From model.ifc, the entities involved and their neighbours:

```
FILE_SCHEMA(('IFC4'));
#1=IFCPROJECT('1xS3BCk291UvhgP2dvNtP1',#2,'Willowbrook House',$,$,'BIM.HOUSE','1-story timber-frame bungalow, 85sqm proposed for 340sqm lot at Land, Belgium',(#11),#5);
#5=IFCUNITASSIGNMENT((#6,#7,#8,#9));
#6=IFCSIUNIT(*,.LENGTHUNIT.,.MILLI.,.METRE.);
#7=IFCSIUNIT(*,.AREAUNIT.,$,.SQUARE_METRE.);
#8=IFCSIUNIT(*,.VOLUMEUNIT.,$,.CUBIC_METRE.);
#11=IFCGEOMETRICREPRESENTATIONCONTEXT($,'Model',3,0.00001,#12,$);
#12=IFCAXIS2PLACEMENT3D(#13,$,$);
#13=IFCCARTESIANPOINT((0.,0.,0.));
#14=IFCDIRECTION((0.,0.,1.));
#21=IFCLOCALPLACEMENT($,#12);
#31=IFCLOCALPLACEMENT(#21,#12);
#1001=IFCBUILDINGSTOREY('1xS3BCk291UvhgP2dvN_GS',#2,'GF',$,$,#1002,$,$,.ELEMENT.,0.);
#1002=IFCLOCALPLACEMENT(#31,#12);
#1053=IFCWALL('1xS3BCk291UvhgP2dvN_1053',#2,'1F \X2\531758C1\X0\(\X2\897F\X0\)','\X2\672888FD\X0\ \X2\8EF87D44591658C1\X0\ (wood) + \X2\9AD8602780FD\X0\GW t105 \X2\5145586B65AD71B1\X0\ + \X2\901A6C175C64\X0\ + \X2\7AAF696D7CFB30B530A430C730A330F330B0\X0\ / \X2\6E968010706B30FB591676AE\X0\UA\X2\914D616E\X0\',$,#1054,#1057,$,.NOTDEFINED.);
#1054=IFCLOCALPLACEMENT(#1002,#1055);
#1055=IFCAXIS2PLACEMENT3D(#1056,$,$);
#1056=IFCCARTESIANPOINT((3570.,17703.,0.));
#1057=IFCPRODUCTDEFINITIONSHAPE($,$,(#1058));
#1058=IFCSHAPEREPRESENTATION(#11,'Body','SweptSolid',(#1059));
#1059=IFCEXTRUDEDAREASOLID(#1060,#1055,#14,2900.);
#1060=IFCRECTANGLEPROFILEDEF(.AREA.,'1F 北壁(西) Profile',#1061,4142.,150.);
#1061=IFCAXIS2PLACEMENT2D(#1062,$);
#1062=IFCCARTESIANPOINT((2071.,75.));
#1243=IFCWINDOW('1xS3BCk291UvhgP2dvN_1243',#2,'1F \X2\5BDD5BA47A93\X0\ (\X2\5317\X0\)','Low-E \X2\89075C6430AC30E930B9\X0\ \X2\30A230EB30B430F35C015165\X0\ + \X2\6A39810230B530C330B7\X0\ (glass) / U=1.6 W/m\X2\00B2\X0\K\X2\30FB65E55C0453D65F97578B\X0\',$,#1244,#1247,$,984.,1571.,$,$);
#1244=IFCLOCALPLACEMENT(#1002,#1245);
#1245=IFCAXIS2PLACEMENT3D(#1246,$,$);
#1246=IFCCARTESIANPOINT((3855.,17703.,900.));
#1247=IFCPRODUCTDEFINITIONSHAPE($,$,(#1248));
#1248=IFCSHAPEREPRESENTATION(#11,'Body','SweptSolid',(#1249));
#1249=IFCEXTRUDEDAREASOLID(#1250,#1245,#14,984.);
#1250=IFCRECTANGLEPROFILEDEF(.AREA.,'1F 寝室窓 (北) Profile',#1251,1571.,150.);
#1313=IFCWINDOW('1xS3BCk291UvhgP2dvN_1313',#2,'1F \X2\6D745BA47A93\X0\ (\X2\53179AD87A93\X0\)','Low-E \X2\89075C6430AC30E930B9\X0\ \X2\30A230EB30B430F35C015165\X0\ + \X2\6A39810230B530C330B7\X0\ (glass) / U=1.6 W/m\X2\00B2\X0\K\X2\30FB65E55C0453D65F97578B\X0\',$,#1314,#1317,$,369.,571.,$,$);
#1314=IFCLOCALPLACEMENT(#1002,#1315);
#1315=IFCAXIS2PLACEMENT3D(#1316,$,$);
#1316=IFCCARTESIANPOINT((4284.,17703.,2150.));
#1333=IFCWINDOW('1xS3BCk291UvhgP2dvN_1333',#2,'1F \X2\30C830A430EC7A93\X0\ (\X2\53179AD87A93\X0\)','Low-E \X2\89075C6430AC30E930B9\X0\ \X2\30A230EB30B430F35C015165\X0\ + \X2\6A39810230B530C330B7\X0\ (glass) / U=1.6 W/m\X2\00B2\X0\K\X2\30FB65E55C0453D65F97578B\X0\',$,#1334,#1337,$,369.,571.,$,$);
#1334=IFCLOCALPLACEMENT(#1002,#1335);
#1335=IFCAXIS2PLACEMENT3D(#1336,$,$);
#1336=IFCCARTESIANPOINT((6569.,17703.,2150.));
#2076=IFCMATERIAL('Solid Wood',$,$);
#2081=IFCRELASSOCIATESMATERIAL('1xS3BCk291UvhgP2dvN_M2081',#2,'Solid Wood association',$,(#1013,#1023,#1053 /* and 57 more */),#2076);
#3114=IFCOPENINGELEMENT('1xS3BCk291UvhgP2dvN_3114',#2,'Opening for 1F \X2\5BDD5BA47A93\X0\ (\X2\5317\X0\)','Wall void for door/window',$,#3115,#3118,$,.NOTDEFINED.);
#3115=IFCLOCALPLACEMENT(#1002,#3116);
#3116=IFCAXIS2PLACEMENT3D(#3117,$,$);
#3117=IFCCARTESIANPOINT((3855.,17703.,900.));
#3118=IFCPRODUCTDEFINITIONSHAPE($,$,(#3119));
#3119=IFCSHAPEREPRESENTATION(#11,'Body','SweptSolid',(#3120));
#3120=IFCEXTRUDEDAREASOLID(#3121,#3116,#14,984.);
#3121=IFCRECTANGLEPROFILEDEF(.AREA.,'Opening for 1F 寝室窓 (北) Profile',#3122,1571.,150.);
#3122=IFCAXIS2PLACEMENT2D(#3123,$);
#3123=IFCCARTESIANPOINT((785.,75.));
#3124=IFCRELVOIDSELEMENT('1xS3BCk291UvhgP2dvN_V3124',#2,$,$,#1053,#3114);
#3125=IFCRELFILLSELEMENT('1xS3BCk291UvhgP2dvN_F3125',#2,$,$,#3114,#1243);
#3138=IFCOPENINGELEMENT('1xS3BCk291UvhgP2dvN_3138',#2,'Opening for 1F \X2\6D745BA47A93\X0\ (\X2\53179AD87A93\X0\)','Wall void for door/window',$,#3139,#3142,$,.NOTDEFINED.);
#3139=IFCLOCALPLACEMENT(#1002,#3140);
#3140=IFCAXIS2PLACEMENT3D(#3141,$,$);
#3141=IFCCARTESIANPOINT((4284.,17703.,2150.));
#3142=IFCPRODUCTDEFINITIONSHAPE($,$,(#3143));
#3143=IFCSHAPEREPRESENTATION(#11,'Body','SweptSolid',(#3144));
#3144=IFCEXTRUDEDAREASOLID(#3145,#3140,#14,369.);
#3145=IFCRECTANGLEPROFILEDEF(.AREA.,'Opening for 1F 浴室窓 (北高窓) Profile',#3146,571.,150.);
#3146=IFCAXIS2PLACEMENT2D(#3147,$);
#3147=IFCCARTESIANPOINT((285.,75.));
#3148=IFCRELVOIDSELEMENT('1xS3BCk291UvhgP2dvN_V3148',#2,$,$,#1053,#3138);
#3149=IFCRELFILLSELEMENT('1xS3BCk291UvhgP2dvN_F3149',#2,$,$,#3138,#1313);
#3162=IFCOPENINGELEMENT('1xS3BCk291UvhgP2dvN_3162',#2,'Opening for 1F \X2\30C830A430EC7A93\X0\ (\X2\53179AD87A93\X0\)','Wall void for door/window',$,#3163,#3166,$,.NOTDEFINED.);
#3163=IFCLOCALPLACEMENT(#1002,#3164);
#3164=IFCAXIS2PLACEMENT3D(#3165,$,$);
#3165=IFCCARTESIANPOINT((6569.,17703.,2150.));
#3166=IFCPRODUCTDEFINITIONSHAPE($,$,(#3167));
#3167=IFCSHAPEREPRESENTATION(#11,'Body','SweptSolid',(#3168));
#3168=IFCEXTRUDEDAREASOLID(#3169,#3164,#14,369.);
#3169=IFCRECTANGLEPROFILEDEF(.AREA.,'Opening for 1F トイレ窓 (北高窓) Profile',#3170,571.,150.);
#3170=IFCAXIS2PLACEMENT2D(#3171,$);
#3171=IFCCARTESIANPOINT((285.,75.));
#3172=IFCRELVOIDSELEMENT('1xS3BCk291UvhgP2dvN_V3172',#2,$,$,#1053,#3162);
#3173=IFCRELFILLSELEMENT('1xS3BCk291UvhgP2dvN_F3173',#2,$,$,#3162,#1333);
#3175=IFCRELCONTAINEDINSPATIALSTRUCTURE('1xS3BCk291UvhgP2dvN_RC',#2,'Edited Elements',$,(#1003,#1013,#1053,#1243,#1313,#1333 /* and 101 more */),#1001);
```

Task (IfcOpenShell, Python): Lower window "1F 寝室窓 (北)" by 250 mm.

```python
import numpy as np
import ifcopenshell
import ifcopenshell.api.geometry
import ifcopenshell.util.placement
import ifcopenshell.util.unit

model = ifcopenshell.open("model.ifc")
unit_scale = ifcopenshell.util.unit.calculate_unit_scale(model)

window = model.by_guid("1xS3BCk291UvhgP2dvN_1243")
opening = window.FillsVoids[0].RelatingOpeningElement
dz = -0.25 / unit_scale

shift = np.array([0.0, 0.0, dz])
# The window is not placed relative to its opening, so move both.
for product in (opening, window):
    matrix = ifcopenshell.util.placement.get_local_placement(product.ObjectPlacement)
    matrix[:3, 3] += shift
    ifcopenshell.api.geometry.edit_object_placement(model, product=product, matrix=matrix, is_si=False)

print(f"moved by {dz * unit_scale:+.3f} m")

model.write("model_v2.ifc")
```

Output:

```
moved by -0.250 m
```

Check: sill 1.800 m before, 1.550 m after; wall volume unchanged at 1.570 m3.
